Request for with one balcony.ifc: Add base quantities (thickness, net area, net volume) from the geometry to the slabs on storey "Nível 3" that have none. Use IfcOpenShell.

First a look at what the model holds.

```python
import ifcopenshell
import ifcopenshell.util.element
import ifcopenshell.util.unit

model = ifcopenshell.open("with one balcony.ifc")
print(model.schema)
for unit_type in ("LENGTHUNIT", "AREAUNIT", "VOLUMEUNIT"):
    print(unit_type, ifcopenshell.util.unit.calculate_unit_scale(model, unit_type))
storey = next(s for s in model.by_type("IfcBuildingStorey") if s.Name == "Nível 3")
slabs = [e for e in ifcopenshell.util.element.get_decomposition(storey) if e.is_a("IfcSlab")]
for e in sorted(slabs, key=lambda e: e.id()):
    print(e.id(), e.is_a(), e.Name, list(ifcopenshell.util.element.get_psets(e, qtos_only=True)), sep=" | ")
```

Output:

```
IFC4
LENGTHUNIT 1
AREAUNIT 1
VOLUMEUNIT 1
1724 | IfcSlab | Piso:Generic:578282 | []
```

```python
import ifcopenshell
import ifcopenshell.api.pset
import ifcopenshell.geom
import ifcopenshell.util.element
import ifcopenshell.util.shape
import ifcopenshell.util.unit

model = ifcopenshell.open("with one balcony.ifc")
unit_scale = ifcopenshell.util.unit.calculate_unit_scale(model)
area_scale = ifcopenshell.util.unit.calculate_unit_scale(model, "AREAUNIT")
volume_scale = ifcopenshell.util.unit.calculate_unit_scale(model, "VOLUMEUNIT")
settings = ifcopenshell.geom.settings()

storey = next(s for s in model.by_type("IfcBuildingStorey") if s.Name == "Nível 3")
slabs = [e for e in ifcopenshell.util.element.get_decomposition(storey) if e.is_a("IfcSlab")]

for e in sorted(slabs, key=lambda e: e.id()):
    if ifcopenshell.util.element.get_psets(e, qtos_only=True, should_inherit=False):
        continue
    # Geometry comes back in metres, in the element's own axes.
    shape = ifcopenshell.geom.create_shape(settings, e)
    values = {
        "Width": ifcopenshell.util.shape.get_z(shape.geometry) / unit_scale,
        "NetArea": ifcopenshell.util.shape.get_footprint_area(shape.geometry) / area_scale,
        "NetVolume": ifcopenshell.util.shape.get_volume(shape.geometry) / volume_scale,
    }
    qto = ifcopenshell.api.pset.add_qto(model, product=e, name="Qto_SlabBaseQuantities")
    ifcopenshell.api.pset.edit_qto(model, qto=qto, properties=values)
    print(e.id(), {k: round(v, 3) for k, v in values.items()})

model.write("with one balcony_updated.ifc")
```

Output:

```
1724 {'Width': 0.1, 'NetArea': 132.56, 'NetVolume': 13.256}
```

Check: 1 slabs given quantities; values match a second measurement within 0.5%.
